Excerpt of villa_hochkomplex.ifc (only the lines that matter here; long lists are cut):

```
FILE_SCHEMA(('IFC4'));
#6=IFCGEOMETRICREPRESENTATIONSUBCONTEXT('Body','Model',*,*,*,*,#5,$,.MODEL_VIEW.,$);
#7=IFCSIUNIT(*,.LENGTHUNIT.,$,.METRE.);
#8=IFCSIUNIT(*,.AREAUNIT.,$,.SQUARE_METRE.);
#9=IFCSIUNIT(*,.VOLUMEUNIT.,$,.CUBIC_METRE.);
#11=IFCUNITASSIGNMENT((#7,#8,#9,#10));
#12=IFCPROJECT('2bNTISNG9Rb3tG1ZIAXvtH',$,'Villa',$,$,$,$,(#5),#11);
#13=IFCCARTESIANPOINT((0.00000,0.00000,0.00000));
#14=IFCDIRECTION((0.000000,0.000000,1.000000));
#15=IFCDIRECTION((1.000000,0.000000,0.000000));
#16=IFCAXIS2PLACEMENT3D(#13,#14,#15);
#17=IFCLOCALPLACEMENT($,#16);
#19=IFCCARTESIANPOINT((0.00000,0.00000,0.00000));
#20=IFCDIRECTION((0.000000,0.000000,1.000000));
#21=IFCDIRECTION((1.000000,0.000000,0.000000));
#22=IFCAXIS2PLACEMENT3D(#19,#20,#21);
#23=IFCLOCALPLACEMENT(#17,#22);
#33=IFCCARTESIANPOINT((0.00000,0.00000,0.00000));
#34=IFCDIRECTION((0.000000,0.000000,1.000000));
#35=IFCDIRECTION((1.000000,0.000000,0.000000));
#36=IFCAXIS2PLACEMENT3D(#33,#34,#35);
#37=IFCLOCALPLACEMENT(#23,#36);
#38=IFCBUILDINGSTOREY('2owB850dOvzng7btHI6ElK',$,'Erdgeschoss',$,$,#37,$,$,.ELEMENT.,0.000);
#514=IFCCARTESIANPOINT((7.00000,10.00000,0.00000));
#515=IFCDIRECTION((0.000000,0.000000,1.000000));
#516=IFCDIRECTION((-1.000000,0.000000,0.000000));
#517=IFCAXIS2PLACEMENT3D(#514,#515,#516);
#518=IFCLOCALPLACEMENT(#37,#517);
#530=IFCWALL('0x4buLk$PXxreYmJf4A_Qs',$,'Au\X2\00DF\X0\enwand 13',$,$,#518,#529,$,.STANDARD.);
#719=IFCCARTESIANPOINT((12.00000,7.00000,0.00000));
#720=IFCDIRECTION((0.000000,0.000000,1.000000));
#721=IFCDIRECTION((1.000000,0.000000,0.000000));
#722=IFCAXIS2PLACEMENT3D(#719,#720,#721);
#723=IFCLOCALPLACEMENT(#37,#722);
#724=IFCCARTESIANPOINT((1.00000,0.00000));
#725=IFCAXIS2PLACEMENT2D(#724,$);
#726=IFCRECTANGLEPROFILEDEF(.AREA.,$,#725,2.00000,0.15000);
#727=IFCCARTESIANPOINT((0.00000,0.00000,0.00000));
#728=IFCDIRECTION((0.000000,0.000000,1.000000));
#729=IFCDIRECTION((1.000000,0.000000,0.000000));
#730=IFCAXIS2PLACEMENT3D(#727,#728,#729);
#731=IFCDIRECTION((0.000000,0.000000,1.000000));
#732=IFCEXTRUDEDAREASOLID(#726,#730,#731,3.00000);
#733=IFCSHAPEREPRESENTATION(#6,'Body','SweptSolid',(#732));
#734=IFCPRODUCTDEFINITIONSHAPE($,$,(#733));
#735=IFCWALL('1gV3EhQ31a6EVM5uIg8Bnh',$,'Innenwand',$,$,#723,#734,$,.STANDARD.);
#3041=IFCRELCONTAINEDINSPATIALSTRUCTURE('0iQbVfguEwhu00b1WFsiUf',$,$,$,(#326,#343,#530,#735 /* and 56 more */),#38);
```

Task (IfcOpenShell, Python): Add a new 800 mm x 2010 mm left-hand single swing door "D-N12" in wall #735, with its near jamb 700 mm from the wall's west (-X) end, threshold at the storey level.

```python
import numpy as np
import ifcopenshell
import ifcopenshell.api.feature
import ifcopenshell.api.geometry
import ifcopenshell.api.root
import ifcopenshell.api.spatial
import ifcopenshell.geom
import ifcopenshell.util.element
import ifcopenshell.util.placement
import ifcopenshell.util.representation
import ifcopenshell.util.shape
import ifcopenshell.util.unit

model = ifcopenshell.open("villa_hochkomplex.ifc")
unit_scale = ifcopenshell.util.unit.calculate_unit_scale(model)
settings = ifcopenshell.geom.settings()


def volume(element):
    """Net volume in cubic metres, openings subtracted."""
    shape = ifcopenshell.geom.create_shape(settings, element)
    return ifcopenshell.util.shape.get_volume(shape.geometry)


wall = model.by_guid("1gV3EhQ31a6EVM5uIg8Bnh")
storey = ifcopenshell.util.element.get_container(wall, ifc_class="IfcBuildingStorey")
context = ifcopenshell.util.representation.get_context(model, "Model", "Body", "MODEL_VIEW")
before = volume(wall)

width, height, from_end, sill = 0.8, 2.01, 0.7, 0.0  # metres

# The wall runs along its own X axis, and the end named is its -X end.
wall_shape = ifcopenshell.geom.create_shape(settings, wall)
x, y, z = ifcopenshell.util.shape.get_vertices(wall_shape.geometry).T
start = x.min() + from_end
face, thickness = float(y.min()), float(y.max() - y.min())
wall_matrix = ifcopenshell.util.placement.get_local_placement(wall.ObjectPlacement)
level = ifcopenshell.util.placement.get_local_placement(storey.ObjectPlacement)[2, 3]


def in_wall(x, y):
    """Placement at x, y metres in the wall's axes, at sill height."""
    matrix = wall_matrix.copy()
    matrix[:, 3] = wall_matrix @ np.array([x / unit_scale, y / unit_scale, 0.0, 1.0])
    matrix[2, 3] = level + sill / unit_scale
    return matrix


# Opening: a box that overshoots both wall faces by 50 mm.
opening = ifcopenshell.api.root.create_entity(model, ifc_class="IfcOpeningElement", predefined_type="OPENING")
box = ifcopenshell.api.geometry.add_wall_representation(
    model, context=context, length=width, height=height, thickness=thickness + 0.1
)
ifcopenshell.api.geometry.assign_representation(model, product=opening, representation=box)
ifcopenshell.api.geometry.edit_object_placement(model, product=opening, matrix=in_wall(start, face - 0.05), is_si=False)
ifcopenshell.api.feature.add_feature(model, feature=opening, element=wall)

door = ifcopenshell.api.root.create_entity(model, ifc_class="IfcDoor", name="D-N12", predefined_type="DOOR")
door.OverallWidth, door.OverallHeight = width / unit_scale, height / unit_scale
door.OperationType = "SINGLE_SWING_LEFT"
body = ifcopenshell.api.geometry.add_door_representation(
    model,
    context=context,
    overall_width=door.OverallWidth,
    overall_height=door.OverallHeight,
    operation_type="SINGLE_SWING_LEFT",
    lining_properties={"LiningDepth": thickness / unit_scale, "ThresholdDepth": thickness / unit_scale},
)
ifcopenshell.api.geometry.assign_representation(model, product=door, representation=body)
ifcopenshell.api.spatial.assign_container(model, products=[door], relating_structure=storey)
ifcopenshell.api.feature.add_filling(model, opening=opening, element=door)

# The lining spans the wall, so the door starts at the wall face.
ifcopenshell.api.geometry.edit_object_placement(model, product=door, matrix=in_wall(start, face), is_si=False)

after = volume(wall)

print(f"wall volume {before:.3f} -> {after:.3f} m3")

model.write("villa_hochkomplex-out.ifc")
```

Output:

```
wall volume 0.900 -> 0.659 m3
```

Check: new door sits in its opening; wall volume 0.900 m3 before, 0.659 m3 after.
